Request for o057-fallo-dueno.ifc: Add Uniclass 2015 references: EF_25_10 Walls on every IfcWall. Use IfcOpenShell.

First a look at what the model holds.

```python
import ifcopenshell

model = ifcopenshell.open("o057-fallo-dueno.ifc")
print(model.schema)
print("classifications:", [c.Name for c in model.by_type("IfcClassification")])
for ifc_class in ("IfcDoor", "IfcRoof", "IfcStair", "IfcWall", "IfcWindow"):
    print(ifc_class, len(model.by_type(ifc_class)))
```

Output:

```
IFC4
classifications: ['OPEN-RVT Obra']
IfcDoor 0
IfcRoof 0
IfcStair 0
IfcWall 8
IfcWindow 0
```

```python
import ifcopenshell
import ifcopenshell.api.classification

model = ifcopenshell.open("o057-fallo-dueno.ifc")

system = ifcopenshell.api.classification.add_classification(model, classification="Uniclass 2015")

codes = {
    "IfcWall": ("EF_25_10", "Walls"),
}
for ifc_class, (code, name) in codes.items():
    products = model.by_type(ifc_class)
    ifcopenshell.api.classification.add_reference(
        model, products=products, classification=system, identification=code, name=name
    )
    print(code, len(products))

model.write("o057-fallo-dueno-out.ifc")
```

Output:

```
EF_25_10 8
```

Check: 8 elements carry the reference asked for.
